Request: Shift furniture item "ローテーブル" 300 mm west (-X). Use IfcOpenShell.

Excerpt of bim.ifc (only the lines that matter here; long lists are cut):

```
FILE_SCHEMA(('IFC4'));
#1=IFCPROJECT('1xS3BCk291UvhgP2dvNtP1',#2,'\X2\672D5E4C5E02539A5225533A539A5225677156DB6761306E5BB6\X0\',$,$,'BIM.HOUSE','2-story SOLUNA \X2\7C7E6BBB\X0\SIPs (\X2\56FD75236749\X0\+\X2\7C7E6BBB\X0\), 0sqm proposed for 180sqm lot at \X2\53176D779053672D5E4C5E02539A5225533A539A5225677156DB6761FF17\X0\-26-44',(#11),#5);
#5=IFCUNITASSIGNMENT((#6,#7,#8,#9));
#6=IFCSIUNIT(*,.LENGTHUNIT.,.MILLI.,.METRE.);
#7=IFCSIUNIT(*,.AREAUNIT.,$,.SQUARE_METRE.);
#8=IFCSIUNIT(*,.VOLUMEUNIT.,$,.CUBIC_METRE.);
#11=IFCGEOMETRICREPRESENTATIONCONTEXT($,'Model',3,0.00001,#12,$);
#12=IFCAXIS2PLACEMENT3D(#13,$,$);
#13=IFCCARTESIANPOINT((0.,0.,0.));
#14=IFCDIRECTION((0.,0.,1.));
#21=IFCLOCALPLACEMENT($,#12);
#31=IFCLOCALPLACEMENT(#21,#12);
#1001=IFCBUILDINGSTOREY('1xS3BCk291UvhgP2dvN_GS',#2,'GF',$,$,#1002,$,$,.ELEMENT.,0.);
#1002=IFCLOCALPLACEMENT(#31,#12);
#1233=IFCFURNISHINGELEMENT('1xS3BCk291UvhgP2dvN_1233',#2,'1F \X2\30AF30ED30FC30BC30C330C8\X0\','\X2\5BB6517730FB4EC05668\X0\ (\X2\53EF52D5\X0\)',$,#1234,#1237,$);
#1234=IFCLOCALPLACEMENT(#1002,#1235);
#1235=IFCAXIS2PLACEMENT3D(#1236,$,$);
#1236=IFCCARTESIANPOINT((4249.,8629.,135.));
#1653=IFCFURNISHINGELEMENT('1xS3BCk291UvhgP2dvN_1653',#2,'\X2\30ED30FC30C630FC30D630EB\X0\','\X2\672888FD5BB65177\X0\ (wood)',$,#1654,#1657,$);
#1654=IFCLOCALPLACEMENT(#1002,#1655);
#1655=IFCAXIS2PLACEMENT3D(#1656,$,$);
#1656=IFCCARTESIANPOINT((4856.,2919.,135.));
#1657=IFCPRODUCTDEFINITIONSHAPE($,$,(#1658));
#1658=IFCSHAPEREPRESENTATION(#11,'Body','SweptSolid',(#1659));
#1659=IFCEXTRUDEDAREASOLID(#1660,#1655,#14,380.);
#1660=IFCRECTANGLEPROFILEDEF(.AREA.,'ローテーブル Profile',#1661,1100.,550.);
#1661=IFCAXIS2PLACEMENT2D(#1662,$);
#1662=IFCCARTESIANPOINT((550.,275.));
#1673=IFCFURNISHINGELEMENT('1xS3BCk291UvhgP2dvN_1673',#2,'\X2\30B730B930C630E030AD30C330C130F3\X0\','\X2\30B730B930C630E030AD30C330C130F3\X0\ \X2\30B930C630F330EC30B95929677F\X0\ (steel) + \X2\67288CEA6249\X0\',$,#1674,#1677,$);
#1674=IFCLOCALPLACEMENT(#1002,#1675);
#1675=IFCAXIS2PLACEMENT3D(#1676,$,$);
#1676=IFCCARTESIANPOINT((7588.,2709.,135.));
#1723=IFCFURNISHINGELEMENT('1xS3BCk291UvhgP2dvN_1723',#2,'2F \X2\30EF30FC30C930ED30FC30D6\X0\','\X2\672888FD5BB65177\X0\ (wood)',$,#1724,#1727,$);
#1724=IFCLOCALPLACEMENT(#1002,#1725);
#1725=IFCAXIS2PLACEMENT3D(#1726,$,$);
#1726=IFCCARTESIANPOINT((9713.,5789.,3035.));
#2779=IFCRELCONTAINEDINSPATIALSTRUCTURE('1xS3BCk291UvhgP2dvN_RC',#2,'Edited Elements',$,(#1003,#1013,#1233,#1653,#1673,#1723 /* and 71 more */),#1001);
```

```python
import ifcopenshell
import ifcopenshell.api.geometry
import ifcopenshell.util.placement
import ifcopenshell.util.unit

model = ifcopenshell.open("bim.ifc")
unit_scale = ifcopenshell.util.unit.calculate_unit_scale(model)

item = model.by_id(1653)
matrix = ifcopenshell.util.placement.get_local_placement(item.ObjectPlacement)
matrix[0, 3] -= 0.3 / unit_scale
ifcopenshell.api.geometry.edit_object_placement(model, product=item, matrix=matrix, is_si=False)

print(ifcopenshell.util.placement.get_local_placement(item.ObjectPlacement).round(3) + 0.0)

model.write("bim_updated.ifc")
```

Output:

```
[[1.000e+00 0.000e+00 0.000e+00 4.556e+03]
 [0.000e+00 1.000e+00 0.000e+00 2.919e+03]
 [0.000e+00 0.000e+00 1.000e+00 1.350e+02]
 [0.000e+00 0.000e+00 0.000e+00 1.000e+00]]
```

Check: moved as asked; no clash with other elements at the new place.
